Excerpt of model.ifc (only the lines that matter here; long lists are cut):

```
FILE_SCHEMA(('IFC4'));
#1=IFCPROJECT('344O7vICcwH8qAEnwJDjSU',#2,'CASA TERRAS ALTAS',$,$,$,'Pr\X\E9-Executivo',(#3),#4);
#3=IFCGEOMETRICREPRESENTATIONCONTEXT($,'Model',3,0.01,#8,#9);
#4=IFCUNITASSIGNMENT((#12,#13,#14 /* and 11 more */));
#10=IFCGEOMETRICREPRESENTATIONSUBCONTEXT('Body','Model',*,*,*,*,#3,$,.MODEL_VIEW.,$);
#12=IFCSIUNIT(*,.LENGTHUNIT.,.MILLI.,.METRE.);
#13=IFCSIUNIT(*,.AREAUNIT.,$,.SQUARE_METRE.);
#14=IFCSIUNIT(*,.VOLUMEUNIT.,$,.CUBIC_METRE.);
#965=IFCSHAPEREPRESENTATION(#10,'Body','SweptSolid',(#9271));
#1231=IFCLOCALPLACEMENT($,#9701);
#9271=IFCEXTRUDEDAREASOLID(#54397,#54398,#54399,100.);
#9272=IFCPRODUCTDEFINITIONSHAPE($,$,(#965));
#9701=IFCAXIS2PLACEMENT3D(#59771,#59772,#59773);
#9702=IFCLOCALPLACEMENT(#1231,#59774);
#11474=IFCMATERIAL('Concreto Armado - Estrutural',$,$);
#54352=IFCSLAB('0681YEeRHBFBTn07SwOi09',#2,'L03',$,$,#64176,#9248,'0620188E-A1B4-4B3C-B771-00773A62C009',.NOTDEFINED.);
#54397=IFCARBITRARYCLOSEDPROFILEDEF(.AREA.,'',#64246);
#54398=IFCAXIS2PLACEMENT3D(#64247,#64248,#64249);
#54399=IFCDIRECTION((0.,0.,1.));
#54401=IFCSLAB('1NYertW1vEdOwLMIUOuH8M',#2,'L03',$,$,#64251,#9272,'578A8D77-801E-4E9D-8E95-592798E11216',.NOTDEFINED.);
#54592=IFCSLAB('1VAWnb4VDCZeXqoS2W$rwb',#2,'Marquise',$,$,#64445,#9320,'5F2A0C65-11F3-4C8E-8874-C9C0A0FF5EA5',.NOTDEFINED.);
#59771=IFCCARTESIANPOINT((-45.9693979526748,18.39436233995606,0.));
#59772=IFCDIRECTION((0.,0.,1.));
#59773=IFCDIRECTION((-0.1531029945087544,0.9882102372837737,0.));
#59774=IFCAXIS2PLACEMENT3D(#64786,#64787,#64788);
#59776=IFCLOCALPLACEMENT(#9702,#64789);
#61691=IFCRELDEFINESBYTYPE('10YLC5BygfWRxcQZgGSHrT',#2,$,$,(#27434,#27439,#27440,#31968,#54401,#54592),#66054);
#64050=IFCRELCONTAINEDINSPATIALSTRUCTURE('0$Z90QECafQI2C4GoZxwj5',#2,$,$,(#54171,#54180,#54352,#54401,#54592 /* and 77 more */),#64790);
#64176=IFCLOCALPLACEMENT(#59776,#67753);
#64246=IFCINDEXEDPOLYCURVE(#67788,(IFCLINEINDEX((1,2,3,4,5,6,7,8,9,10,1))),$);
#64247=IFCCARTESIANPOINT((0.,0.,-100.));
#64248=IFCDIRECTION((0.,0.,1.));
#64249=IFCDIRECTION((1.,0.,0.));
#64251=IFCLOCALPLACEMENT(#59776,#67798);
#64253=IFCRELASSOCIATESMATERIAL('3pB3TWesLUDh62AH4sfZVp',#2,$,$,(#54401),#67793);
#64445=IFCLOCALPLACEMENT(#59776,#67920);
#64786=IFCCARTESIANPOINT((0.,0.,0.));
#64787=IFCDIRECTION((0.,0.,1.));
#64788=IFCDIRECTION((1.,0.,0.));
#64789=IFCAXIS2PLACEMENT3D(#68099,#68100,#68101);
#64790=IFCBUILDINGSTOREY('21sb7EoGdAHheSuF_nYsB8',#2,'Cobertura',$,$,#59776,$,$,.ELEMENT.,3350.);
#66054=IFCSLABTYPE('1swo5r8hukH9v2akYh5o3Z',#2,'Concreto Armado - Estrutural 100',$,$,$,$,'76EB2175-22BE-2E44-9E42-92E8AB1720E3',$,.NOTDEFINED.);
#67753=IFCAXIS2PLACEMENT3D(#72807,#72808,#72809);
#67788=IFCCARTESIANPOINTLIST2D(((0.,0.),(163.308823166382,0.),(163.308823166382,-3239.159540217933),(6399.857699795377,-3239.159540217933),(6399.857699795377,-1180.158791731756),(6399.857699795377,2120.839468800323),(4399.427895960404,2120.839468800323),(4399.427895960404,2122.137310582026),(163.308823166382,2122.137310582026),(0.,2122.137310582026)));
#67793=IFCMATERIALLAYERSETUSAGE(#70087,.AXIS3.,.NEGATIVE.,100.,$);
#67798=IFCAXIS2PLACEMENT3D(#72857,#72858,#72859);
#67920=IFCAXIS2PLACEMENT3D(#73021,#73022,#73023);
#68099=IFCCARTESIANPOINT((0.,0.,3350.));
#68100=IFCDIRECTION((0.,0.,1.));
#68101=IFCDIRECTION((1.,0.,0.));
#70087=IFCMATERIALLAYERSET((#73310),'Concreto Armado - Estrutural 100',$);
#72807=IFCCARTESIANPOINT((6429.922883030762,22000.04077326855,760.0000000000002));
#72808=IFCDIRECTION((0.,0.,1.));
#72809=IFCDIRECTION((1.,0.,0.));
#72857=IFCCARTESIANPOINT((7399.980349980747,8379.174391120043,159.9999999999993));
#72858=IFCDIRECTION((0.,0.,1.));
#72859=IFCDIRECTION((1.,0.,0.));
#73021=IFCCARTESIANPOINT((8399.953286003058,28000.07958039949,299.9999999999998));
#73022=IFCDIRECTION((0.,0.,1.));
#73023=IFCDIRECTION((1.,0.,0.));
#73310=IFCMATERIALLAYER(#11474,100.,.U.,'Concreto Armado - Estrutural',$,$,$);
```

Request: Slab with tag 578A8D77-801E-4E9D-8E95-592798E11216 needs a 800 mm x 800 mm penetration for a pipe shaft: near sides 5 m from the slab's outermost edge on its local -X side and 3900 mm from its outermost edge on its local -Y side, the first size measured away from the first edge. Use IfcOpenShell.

```python
import numpy as np
import ifcopenshell
import ifcopenshell.api.feature
import ifcopenshell.api.geometry
import ifcopenshell.api.root
import ifcopenshell.geom
import ifcopenshell.util.placement
import ifcopenshell.util.representation
import ifcopenshell.util.shape
import ifcopenshell.util.unit

model = ifcopenshell.open("model.ifc")
unit_scale = ifcopenshell.util.unit.calculate_unit_scale(model)
settings = ifcopenshell.geom.settings()


def volume(element):
    """Net volume in cubic metres, openings subtracted."""
    shape = ifcopenshell.geom.create_shape(settings, element)
    return ifcopenshell.util.shape.get_volume(shape.geometry)


slab = model.by_guid("1NYertW1vEdOwLMIUOuH8M")
before = volume(slab)

# Extent in the slab's own axes, in metres. The edges named are its -X and -Y sides.
slab_shape = ifcopenshell.geom.create_shape(settings, slab)
vertices = ifcopenshell.util.shape.get_vertices(slab_shape.geometry)
x_min, y_min, bottom = vertices.min(axis=0)
top = vertices[:, 2].max()

opening = ifcopenshell.api.root.create_entity(model, ifc_class="IfcOpeningElement", name="Pipe shaft opening", predefined_type="OPENING")
context = ifcopenshell.util.representation.get_context(model, "Model", "Body", "MODEL_VIEW")
width, depth = 0.8, 0.8
outline = [(0.0, 0.0), (width, 0.0), (width, depth), (0.0, depth), (0.0, 0.0)]
# Overshoot both faces by 50 mm so the cut is clean.
shape = ifcopenshell.api.geometry.add_slab_representation(
    model, context=context, depth=top - bottom + 0.1, polyline=outline
)
ifcopenshell.api.geometry.assign_representation(model, product=opening, representation=shape)

matrix = ifcopenshell.util.placement.get_local_placement(slab.ObjectPlacement)
matrix[:, 3] = matrix @ np.append(np.array([x_min + 5, y_min + 3.9, bottom - 0.05]) / unit_scale, 1.0)
ifcopenshell.api.geometry.edit_object_placement(model, product=opening, matrix=matrix, is_si=False)
ifcopenshell.api.feature.add_feature(model, feature=opening, element=slab)

after = volume(slab)

print(f"slab volume {before:.3f} -> {after:.3f} m3")

model.write("model_rev.ifc")
```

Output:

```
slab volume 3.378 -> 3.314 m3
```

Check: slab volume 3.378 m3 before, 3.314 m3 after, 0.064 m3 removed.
